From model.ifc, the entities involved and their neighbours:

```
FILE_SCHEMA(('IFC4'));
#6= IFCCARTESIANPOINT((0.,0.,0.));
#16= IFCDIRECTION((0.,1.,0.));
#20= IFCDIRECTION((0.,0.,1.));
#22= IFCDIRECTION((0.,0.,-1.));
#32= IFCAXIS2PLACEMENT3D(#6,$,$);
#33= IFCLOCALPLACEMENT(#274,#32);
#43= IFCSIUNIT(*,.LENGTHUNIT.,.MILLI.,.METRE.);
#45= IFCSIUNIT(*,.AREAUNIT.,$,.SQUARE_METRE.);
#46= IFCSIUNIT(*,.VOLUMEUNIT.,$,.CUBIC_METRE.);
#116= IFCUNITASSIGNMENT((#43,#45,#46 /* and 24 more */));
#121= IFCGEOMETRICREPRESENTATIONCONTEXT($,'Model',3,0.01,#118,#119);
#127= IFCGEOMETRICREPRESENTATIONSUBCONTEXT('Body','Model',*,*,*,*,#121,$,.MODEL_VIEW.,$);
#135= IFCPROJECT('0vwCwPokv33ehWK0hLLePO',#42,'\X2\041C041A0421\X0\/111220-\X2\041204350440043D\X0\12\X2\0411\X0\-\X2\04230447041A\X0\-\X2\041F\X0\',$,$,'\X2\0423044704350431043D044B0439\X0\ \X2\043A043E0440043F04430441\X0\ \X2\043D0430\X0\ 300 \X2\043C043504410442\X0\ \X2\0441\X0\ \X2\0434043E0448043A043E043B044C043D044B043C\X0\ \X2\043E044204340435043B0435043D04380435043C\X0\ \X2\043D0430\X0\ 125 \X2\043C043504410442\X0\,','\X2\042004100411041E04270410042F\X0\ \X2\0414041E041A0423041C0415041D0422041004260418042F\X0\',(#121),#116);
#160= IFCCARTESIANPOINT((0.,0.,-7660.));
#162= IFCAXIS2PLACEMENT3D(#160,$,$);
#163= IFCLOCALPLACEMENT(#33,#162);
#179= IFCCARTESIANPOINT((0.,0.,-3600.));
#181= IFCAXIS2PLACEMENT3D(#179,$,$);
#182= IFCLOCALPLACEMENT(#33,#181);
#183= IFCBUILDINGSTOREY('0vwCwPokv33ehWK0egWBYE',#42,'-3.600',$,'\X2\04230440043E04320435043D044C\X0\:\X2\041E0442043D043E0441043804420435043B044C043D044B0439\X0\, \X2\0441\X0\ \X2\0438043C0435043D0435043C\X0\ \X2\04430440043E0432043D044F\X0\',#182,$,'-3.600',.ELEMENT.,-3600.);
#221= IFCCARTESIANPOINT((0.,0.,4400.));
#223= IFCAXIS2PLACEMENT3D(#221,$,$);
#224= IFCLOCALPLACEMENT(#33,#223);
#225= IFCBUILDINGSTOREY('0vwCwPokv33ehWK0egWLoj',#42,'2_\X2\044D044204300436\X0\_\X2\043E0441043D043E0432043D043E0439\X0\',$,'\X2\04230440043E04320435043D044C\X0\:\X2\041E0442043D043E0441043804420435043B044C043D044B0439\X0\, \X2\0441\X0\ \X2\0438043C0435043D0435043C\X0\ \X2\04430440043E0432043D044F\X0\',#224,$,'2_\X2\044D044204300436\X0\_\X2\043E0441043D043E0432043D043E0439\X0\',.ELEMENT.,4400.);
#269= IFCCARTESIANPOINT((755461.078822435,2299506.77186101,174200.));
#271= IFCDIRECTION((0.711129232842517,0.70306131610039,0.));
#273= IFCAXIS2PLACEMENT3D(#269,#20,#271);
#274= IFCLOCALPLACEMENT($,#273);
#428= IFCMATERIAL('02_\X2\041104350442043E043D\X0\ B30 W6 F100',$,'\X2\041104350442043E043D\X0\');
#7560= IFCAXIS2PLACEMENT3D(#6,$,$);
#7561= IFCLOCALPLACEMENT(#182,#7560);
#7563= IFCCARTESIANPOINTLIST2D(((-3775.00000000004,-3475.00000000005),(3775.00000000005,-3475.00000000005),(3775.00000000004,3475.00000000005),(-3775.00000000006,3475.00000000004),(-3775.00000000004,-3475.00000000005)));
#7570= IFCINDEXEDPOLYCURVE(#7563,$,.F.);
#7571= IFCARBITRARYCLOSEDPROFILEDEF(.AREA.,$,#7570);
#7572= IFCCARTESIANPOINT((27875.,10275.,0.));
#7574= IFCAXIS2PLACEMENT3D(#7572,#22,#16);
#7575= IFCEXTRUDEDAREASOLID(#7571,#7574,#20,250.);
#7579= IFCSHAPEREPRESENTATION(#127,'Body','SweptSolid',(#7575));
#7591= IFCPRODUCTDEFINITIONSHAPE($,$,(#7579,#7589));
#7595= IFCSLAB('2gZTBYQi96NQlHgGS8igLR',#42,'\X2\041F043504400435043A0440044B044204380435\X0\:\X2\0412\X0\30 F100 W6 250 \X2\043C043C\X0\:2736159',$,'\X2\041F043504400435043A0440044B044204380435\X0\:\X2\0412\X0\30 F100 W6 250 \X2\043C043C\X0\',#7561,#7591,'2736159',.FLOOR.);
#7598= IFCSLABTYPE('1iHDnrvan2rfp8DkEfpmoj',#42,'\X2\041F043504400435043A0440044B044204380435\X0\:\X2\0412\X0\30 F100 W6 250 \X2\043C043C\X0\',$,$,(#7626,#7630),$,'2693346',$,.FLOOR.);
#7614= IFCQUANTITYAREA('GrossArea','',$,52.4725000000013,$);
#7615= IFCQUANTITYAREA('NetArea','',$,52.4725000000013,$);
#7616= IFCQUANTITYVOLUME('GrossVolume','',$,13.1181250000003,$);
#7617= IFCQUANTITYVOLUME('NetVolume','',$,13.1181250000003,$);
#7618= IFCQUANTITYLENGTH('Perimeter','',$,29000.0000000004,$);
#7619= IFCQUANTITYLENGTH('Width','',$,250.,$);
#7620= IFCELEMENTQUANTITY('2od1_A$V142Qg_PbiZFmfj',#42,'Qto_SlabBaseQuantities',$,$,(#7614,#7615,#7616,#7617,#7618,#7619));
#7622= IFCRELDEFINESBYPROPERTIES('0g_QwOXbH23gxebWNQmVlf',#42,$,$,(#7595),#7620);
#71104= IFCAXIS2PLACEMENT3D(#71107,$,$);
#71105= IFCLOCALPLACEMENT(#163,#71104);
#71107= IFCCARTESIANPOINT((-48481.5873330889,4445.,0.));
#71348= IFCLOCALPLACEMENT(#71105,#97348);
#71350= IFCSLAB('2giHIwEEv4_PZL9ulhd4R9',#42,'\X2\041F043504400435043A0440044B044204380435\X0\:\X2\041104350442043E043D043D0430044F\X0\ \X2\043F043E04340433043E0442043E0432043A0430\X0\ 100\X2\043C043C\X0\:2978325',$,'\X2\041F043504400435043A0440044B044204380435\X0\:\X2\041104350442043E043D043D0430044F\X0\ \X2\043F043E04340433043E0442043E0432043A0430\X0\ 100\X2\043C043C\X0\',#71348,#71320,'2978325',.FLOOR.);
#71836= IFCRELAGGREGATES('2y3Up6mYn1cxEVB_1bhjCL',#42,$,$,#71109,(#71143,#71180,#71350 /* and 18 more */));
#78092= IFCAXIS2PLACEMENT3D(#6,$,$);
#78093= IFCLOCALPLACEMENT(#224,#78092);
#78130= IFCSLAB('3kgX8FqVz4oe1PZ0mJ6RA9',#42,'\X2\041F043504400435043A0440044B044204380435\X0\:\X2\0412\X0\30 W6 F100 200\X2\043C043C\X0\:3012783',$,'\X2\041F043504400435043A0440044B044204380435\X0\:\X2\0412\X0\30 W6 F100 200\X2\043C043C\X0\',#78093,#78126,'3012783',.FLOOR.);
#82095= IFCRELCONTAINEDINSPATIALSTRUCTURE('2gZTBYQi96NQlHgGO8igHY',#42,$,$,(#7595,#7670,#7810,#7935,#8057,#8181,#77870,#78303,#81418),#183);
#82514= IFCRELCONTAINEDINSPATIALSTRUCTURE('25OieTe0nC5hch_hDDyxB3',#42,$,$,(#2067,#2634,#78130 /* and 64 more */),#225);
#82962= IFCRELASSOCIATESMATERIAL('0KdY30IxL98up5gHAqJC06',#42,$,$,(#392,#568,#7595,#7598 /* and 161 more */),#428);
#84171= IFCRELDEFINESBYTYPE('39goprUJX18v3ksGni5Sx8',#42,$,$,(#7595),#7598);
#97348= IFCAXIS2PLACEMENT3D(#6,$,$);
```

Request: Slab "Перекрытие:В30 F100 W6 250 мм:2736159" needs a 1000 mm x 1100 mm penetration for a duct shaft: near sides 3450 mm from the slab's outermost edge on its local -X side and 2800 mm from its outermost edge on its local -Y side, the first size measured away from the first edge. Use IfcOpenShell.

```python
import numpy as np
import ifcopenshell
import ifcopenshell.api.feature
import ifcopenshell.api.geometry
import ifcopenshell.api.pset
import ifcopenshell.api.root
import ifcopenshell.geom
import ifcopenshell.util.element
import ifcopenshell.util.placement
import ifcopenshell.util.representation
import ifcopenshell.util.shape
import ifcopenshell.util.unit

model = ifcopenshell.open("model.ifc")
unit_scale = ifcopenshell.util.unit.calculate_unit_scale(model)
area_scale = ifcopenshell.util.unit.calculate_unit_scale(model, "AREAUNIT")
volume_scale = ifcopenshell.util.unit.calculate_unit_scale(model, "VOLUMEUNIT")
settings = ifcopenshell.geom.settings()


def volume(element):
    """Net volume in cubic metres, openings subtracted."""
    shape = ifcopenshell.geom.create_shape(settings, element)
    return ifcopenshell.util.shape.get_volume(shape.geometry)


slab = model.by_guid("2gZTBYQi96NQlHgGS8igLR")
before = volume(slab)

# Extent in the slab's own axes, in metres. The edges named are its -X and -Y sides.
slab_shape = ifcopenshell.geom.create_shape(settings, slab)
vertices = ifcopenshell.util.shape.get_vertices(slab_shape.geometry)
x_min, y_min, bottom = vertices.min(axis=0)
top = vertices[:, 2].max()

opening = ifcopenshell.api.root.create_entity(model, ifc_class="IfcOpeningElement", name="Duct shaft opening", predefined_type="OPENING")
context = ifcopenshell.util.representation.get_context(model, "Model", "Body", "MODEL_VIEW")
width, depth = 1, 1.1
outline = [(0.0, 0.0), (width, 0.0), (width, depth), (0.0, depth), (0.0, 0.0)]
# Overshoot both faces by 50 mm so the cut is clean.
shape = ifcopenshell.api.geometry.add_slab_representation(
    model, context=context, depth=top - bottom + 0.1, polyline=outline
)
ifcopenshell.api.geometry.assign_representation(model, product=opening, representation=shape)

matrix = ifcopenshell.util.placement.get_local_placement(slab.ObjectPlacement)
matrix[:, 3] = matrix @ np.append(np.array([x_min + 3.45, y_min + 2.8, bottom - 0.05]) / unit_scale, 1.0)
ifcopenshell.api.geometry.edit_object_placement(model, product=opening, matrix=matrix, is_si=False)
ifcopenshell.api.feature.add_feature(model, feature=opening, element=slab)

after = volume(slab)

# Update the slab's stored quantities.
qto = model.by_id(ifcopenshell.util.element.get_pset(slab, "Qto_SlabBaseQuantities", should_inherit=False)["id"])
ifcopenshell.api.pset.edit_qto(model, qto=qto, properties={
    "NetArea": after / (top - bottom) / area_scale,
    "NetVolume": after / volume_scale,
})

print(f"slab volume {before:.3f} -> {after:.3f} m3")

model.write("model_edited.ifc")
```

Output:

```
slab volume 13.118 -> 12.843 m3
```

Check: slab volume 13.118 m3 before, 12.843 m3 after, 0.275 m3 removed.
